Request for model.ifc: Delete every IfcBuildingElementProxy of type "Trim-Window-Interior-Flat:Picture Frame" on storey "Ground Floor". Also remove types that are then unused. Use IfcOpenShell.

First a look at what the model holds.

```python
import ifcopenshell
import ifcopenshell.util.element

model = ifcopenshell.open("model.ifc")
print(model.schema)
storey = next(s for s in model.by_type("IfcBuildingStorey") if s.Name == "Ground Floor")
proxies = [e for e in ifcopenshell.util.element.get_decomposition(storey) if e.is_a("IfcBuildingElementProxy")]
seen = {}
for e in proxies:
    element_type = ifcopenshell.util.element.get_type(e)
    name = element_type.Name if element_type not in (None, e) else None
    seen[name] = seen.get(name, 0) + 1
for name, count in sorted(seen.items(), key=str):
    print(count, "x", name)
```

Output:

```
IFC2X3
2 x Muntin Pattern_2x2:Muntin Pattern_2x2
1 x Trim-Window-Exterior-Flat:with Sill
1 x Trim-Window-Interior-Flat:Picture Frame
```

```python
import ifcopenshell
import ifcopenshell.api.root
import ifcopenshell.util.element

model = ifcopenshell.open("model.ifc")

storey = next(s for s in model.by_type("IfcBuildingStorey") if s.Name == "Ground Floor")
proxies = [e for e in ifcopenshell.util.element.get_decomposition(storey) if e.is_a("IfcBuildingElementProxy")]
targets = [e for e in proxies if (t := ifcopenshell.util.element.get_type(e)) not in (None, e) and t.Name == "Trim-Window-Interior-Flat:Picture Frame"]
types = {ifcopenshell.util.element.get_type(e) for e in targets} - {None, *targets}

for e in targets:
    ifcopenshell.api.root.remove_product(model, product=e)
print(len(targets), "removed")

unused = [t for t in types if not ifcopenshell.util.element.get_types(t)]
for t in unused:
    ifcopenshell.api.root.remove_product(model, product=t)
print(len(unused), "unused types removed")

model.write("model_v2.ifc")
```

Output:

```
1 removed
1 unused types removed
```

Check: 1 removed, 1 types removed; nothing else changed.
